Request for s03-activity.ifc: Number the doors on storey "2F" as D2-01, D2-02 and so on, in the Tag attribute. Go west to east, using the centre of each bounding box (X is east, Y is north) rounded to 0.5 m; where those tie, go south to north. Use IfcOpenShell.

First a look at what the model holds.

```python
import ifcopenshell
import ifcopenshell.util.element
import ifcopenshell.util.placement

model = ifcopenshell.open("s03-activity.ifc")
print(model.schema)
storey = next(s for s in model.by_type("IfcBuildingStorey") if s.Name == "2F")
doors = [e for e in ifcopenshell.util.element.get_decomposition(storey) if e.is_a("IfcDoor")]
for e in sorted(doors, key=lambda e: e.id()):
    origin = ifcopenshell.util.placement.get_local_placement(e.ObjectPlacement)[:3, 3]
    print(e.id(), e.Tag, e.Name, origin.round(2) + 0.0, sep=" | ")
```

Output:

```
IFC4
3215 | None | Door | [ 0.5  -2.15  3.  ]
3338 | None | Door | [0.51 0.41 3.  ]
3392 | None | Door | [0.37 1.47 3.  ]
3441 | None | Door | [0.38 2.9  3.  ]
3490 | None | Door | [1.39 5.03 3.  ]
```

```python
import ifcopenshell
import ifcopenshell.geom
import ifcopenshell.util.element
import ifcopenshell.util.shape

model = ifcopenshell.open("s03-activity.ifc")
settings = ifcopenshell.geom.settings()
settings.set("use-world-coords", True)


def centre(element):
    shape = ifcopenshell.geom.create_shape(settings, element)
    return ifcopenshell.util.shape.get_bbox_centroid(shape.geometry)


storey = next(s for s in model.by_type("IfcBuildingStorey") if s.Name == "2F")
doors = [e for e in ifcopenshell.util.element.get_decomposition(storey) if e.is_a("IfcDoor")]

# Insertion points can sit at a corner or the storey origin, so sort by the geometry (in metres).
centres = {e: centre(e) for e in doors}
doors.sort(key=lambda e: (round(centres[e][0] / 0.5), centres[e][1]))

for i, e in enumerate(doors, start=1):
    number = f"D2-{i:02d}"
    e.Tag = number
    print(e.id(), number)

model.write("s03-activity_updated.ifc")
```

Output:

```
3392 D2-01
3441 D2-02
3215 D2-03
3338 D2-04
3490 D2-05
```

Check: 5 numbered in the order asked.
